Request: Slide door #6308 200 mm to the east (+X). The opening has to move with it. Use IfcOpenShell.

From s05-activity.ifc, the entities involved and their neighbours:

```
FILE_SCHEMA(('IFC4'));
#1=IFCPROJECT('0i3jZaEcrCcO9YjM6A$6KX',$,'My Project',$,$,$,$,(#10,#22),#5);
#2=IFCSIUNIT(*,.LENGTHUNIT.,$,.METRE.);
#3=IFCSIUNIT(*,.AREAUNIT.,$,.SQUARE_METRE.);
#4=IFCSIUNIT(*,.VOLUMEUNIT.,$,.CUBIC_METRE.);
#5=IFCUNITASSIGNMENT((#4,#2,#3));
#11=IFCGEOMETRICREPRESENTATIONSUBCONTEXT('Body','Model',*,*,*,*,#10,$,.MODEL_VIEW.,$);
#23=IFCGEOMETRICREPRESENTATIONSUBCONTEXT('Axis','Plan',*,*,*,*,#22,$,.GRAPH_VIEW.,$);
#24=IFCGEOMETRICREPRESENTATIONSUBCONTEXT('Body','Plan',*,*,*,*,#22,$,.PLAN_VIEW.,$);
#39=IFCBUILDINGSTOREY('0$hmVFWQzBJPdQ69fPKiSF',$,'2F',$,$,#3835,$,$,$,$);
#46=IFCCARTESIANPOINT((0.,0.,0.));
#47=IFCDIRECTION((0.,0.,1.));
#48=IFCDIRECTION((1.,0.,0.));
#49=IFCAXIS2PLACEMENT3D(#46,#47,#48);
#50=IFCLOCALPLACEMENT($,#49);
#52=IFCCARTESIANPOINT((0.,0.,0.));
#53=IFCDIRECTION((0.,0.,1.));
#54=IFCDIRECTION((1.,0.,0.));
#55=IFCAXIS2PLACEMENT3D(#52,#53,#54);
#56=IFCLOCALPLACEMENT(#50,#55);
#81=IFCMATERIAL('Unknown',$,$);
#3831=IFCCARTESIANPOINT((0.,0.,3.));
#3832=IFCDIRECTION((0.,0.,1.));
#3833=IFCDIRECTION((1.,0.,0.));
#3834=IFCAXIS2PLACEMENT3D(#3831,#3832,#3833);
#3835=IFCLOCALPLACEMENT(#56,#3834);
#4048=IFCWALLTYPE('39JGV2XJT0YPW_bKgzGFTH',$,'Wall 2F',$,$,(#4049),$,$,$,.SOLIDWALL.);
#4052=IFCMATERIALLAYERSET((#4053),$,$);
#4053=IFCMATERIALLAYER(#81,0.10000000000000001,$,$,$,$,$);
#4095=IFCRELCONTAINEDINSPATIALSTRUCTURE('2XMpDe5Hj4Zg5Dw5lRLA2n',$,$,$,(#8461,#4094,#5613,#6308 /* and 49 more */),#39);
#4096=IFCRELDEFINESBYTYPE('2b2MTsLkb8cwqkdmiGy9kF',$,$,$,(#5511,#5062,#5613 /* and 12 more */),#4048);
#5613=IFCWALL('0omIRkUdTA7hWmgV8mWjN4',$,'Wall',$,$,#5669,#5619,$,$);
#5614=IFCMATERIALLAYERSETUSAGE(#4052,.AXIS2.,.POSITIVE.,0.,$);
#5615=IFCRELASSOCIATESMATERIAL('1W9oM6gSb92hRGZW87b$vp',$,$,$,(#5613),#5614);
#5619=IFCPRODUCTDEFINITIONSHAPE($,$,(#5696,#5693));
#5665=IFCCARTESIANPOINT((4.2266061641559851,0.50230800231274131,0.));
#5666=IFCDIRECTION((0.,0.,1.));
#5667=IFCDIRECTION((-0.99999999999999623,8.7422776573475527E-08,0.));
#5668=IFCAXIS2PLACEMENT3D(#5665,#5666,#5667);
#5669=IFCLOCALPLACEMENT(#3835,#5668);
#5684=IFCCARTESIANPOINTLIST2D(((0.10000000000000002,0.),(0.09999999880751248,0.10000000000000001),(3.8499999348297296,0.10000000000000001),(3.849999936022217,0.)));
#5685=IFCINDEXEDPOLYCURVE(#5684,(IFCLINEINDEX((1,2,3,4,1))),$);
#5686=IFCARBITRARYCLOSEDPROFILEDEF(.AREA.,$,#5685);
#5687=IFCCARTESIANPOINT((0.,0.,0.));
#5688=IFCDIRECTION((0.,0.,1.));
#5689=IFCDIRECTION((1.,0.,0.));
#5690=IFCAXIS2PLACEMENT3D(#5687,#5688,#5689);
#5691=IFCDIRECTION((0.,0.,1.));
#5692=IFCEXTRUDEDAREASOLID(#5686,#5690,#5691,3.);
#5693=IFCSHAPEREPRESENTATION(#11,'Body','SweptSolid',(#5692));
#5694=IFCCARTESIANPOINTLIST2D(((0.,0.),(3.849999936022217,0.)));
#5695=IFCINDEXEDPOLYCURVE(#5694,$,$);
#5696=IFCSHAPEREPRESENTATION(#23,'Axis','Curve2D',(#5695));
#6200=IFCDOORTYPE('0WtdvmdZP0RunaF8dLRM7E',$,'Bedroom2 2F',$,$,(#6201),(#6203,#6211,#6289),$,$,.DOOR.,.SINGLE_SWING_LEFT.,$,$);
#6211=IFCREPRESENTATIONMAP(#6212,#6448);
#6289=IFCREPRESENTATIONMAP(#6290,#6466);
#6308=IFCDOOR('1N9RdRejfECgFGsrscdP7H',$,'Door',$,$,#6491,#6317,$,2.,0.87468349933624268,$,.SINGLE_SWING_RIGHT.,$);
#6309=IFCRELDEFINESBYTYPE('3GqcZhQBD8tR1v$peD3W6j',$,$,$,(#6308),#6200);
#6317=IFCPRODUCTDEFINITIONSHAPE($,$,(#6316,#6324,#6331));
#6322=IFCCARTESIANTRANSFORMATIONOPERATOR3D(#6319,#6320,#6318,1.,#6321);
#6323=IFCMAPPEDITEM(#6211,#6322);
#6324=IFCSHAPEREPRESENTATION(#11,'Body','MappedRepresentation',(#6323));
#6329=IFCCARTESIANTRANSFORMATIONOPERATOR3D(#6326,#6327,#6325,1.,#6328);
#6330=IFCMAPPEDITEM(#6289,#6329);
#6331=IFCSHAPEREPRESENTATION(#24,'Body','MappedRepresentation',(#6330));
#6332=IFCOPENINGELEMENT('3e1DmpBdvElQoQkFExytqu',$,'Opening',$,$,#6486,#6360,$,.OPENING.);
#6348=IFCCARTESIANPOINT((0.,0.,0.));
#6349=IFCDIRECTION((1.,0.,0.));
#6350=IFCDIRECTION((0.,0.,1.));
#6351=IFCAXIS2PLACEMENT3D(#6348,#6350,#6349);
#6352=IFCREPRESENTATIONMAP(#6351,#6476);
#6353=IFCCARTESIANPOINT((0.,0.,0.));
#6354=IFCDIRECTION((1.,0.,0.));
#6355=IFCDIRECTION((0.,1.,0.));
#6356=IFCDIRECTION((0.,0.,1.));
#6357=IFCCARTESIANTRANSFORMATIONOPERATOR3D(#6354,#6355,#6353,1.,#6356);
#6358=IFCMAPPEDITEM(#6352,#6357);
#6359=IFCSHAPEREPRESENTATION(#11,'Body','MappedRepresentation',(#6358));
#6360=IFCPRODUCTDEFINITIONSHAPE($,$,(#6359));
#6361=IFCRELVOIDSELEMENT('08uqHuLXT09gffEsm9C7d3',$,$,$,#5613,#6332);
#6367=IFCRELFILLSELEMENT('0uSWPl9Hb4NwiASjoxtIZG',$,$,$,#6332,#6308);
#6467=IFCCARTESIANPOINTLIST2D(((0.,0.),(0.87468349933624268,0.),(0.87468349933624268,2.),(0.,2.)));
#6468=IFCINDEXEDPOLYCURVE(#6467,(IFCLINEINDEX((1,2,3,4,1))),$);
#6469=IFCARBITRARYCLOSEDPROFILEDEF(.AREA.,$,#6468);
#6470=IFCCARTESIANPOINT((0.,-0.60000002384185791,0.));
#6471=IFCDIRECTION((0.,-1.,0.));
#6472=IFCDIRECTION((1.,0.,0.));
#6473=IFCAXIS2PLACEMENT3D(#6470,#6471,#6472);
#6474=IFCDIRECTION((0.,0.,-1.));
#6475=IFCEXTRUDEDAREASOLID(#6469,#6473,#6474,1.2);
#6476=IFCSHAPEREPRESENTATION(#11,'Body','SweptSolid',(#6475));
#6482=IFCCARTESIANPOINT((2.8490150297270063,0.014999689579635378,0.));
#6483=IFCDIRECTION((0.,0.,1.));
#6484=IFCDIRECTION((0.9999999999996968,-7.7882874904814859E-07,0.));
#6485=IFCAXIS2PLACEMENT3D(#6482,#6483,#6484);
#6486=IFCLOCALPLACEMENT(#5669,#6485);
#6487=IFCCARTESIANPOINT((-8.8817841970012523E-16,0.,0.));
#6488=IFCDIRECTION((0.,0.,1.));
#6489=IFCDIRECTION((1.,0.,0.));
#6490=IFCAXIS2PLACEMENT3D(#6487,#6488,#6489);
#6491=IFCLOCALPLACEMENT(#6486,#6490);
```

```python
import ifcopenshell
import ifcopenshell.api.geometry
import ifcopenshell.util.placement
import ifcopenshell.util.unit

model = ifcopenshell.open("s05-activity.ifc")
unit_scale = ifcopenshell.util.unit.calculate_unit_scale(model)

door = model.by_guid("1N9RdRejfECgFGsrscdP7H")
opening = door.FillsVoids[0].RelatingOpeningElement
wall = opening.VoidsElements[0].RelatingBuildingElement

wall_matrix = ifcopenshell.util.placement.get_local_placement(wall.ObjectPlacement)
shift = wall_matrix[:3, 0] * -0.2 / unit_scale
before = ifcopenshell.util.placement.get_local_placement(door.ObjectPlacement)[:3, 3].copy()

# The door is placed relative to its opening, so it follows when the opening moves.
matrix = ifcopenshell.util.placement.get_local_placement(opening.ObjectPlacement)
matrix[:3, 3] += shift
ifcopenshell.api.geometry.edit_object_placement(
    model, product=opening, matrix=matrix, is_si=False, should_transform_children=True
)

after = ifcopenshell.util.placement.get_local_placement(door.ObjectPlacement)[:3, 3]
print("door moved by", (after - before).round(3) + 0.0)

model.write("s05-activity_v2.ifc")
```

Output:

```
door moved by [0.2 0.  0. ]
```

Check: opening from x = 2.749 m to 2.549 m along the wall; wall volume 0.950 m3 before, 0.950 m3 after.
